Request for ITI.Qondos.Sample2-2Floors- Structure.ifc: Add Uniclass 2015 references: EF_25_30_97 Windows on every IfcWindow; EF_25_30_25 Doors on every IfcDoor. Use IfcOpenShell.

First a look at what the model holds.

```python
import ifcopenshell

model = ifcopenshell.open("ITI.Qondos.Sample2-2Floors- Structure.ifc")
print(model.schema)
print("classifications:", [c.Name for c in model.by_type("IfcClassification")])
for ifc_class in ("IfcDoor", "IfcRoof", "IfcStair", "IfcWall", "IfcWindow"):
    print(ifc_class, len(model.by_type(ifc_class)))
```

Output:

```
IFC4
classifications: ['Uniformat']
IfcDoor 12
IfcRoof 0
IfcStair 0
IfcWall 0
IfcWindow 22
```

```python
import ifcopenshell
import ifcopenshell.api.classification

model = ifcopenshell.open("ITI.Qondos.Sample2-2Floors- Structure.ifc")

system = ifcopenshell.api.classification.add_classification(model, classification="Uniclass 2015")

codes = {
    "IfcWindow": ("EF_25_30_97", "Windows"),
    "IfcDoor": ("EF_25_30_25", "Doors"),
}
for ifc_class, (code, name) in codes.items():
    products = model.by_type(ifc_class)
    ifcopenshell.api.classification.add_reference(
        model, products=products, classification=system, identification=code, name=name
    )
    print(code, len(products))

model.write("ITI.Qondos.Sample2-2Floors- Structure_updated.ifc")
```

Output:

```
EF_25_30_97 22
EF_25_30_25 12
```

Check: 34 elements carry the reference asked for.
